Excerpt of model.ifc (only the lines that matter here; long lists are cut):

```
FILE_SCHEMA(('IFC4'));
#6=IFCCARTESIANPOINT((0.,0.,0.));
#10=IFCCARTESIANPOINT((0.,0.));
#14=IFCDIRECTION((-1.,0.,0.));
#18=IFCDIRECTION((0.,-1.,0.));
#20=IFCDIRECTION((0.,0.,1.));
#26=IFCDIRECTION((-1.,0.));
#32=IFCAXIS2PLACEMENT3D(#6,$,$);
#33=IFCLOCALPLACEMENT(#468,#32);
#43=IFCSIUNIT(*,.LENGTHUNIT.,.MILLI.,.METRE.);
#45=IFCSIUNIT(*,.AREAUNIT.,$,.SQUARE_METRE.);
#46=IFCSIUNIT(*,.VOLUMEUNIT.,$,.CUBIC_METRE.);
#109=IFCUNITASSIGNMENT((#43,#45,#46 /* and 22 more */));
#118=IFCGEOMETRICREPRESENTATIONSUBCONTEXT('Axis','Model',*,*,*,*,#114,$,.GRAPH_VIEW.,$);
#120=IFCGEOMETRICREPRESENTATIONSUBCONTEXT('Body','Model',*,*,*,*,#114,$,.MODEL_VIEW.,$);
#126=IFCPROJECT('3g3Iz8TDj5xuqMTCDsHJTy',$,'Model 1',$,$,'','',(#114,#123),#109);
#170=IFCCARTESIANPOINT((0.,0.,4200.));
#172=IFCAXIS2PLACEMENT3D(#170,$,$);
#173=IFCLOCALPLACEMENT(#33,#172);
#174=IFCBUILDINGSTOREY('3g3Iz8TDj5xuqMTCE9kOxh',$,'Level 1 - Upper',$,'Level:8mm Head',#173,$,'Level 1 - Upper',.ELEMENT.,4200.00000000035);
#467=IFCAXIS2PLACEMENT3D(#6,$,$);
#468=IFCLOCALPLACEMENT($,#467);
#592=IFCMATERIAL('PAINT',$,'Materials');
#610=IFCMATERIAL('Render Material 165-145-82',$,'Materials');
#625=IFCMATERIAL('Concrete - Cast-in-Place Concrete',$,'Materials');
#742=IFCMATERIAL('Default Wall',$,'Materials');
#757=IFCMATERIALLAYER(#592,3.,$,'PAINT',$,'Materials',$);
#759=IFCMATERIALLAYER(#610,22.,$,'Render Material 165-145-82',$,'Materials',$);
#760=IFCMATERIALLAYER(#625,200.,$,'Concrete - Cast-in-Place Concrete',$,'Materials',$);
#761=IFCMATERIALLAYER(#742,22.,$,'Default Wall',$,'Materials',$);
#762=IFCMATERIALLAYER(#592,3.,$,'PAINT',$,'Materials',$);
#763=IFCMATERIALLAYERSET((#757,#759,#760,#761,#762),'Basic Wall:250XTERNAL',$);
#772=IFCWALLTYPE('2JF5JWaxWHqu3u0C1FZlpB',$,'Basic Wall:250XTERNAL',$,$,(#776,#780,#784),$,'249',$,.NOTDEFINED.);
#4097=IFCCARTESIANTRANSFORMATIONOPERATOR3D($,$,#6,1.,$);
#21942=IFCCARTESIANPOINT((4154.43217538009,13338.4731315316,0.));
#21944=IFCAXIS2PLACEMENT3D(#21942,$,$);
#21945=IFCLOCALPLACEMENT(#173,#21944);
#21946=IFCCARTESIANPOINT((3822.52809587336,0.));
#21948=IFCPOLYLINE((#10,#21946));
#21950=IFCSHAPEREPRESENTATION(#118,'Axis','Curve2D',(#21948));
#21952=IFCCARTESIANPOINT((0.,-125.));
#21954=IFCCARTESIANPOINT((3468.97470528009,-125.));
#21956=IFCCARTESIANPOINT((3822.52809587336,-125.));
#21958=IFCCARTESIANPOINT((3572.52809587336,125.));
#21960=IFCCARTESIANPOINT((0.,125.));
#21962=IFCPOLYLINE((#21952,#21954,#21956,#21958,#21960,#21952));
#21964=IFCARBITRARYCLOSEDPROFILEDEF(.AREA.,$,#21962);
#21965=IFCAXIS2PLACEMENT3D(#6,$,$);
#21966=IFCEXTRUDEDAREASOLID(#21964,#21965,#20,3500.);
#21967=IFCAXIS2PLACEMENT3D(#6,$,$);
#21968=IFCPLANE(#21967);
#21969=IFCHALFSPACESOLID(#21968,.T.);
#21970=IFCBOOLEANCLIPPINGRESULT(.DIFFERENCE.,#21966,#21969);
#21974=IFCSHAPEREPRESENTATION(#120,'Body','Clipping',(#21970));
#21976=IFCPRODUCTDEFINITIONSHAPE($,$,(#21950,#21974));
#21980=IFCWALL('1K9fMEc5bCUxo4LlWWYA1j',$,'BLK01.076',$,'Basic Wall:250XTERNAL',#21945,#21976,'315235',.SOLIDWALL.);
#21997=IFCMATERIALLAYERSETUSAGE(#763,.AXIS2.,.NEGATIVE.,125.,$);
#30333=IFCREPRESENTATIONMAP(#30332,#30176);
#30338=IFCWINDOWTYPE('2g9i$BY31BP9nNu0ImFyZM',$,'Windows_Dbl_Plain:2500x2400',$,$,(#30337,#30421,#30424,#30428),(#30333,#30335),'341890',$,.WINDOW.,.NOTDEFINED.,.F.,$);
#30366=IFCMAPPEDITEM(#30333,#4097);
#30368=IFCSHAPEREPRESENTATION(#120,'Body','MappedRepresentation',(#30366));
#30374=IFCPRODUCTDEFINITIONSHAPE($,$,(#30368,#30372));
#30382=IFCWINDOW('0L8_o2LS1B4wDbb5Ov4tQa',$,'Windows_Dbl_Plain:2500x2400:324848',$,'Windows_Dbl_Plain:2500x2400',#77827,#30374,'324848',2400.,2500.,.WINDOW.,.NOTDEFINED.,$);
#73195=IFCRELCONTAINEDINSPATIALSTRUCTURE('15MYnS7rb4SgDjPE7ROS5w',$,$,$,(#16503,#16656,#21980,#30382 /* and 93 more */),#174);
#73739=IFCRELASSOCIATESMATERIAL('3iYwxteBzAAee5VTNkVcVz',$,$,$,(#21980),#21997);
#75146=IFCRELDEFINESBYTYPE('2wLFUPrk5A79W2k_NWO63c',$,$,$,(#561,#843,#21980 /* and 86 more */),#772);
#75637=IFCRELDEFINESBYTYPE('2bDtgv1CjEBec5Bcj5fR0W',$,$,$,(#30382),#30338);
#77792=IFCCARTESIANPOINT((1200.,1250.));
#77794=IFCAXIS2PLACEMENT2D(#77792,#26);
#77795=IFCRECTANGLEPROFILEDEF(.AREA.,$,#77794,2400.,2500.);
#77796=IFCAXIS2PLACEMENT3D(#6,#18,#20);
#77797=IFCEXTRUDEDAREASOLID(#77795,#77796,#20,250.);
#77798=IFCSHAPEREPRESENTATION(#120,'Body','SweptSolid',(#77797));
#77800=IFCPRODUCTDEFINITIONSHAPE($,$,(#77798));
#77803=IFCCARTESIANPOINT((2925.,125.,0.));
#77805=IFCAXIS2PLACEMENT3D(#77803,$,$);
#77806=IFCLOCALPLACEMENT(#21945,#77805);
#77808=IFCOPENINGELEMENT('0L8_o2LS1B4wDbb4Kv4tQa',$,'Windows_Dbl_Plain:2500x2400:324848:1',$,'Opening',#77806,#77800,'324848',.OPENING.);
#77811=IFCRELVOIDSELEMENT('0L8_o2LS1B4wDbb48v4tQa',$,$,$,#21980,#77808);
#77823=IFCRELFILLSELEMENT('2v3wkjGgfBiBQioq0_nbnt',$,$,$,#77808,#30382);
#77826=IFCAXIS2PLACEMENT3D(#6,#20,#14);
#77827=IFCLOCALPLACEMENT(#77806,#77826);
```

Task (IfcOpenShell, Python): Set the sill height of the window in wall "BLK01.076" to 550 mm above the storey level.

```python
import numpy as np
import ifcopenshell
import ifcopenshell.api.geometry
import ifcopenshell.geom
import ifcopenshell.util.element
import ifcopenshell.util.placement
import ifcopenshell.util.shape
import ifcopenshell.util.unit

model = ifcopenshell.open("model.ifc")
unit_scale = ifcopenshell.util.unit.calculate_unit_scale(model)

window = model.by_guid("0L8_o2LS1B4wDbb5Ov4tQa")
opening = window.FillsVoids[0].RelatingOpeningElement
storey = ifcopenshell.util.element.get_container(window, ifc_class="IfcBuildingStorey")
level = ifcopenshell.util.placement.get_local_placement(storey.ObjectPlacement)[2, 3]

# The opening's origin need not be at the sill, so measure its lowest point.
shape = ifcopenshell.geom.create_shape(ifcopenshell.geom.settings(), opening)
bottom = ifcopenshell.util.shape.get_shape_bottom_elevation(shape, shape.geometry) / unit_scale
dz = level + 0.55 / unit_scale - bottom

shift = np.array([0.0, 0.0, dz])
# The window is placed relative to its opening, so it follows when the opening moves.
matrix = ifcopenshell.util.placement.get_local_placement(opening.ObjectPlacement)
matrix[:3, 3] += shift
ifcopenshell.api.geometry.edit_object_placement(
    model, product=opening, matrix=matrix, is_si=False, should_transform_children=True
)

print(f"moved by {dz * unit_scale:+.3f} m")

model.write("model-out.ifc")
```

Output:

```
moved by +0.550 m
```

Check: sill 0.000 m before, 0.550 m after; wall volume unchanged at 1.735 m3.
